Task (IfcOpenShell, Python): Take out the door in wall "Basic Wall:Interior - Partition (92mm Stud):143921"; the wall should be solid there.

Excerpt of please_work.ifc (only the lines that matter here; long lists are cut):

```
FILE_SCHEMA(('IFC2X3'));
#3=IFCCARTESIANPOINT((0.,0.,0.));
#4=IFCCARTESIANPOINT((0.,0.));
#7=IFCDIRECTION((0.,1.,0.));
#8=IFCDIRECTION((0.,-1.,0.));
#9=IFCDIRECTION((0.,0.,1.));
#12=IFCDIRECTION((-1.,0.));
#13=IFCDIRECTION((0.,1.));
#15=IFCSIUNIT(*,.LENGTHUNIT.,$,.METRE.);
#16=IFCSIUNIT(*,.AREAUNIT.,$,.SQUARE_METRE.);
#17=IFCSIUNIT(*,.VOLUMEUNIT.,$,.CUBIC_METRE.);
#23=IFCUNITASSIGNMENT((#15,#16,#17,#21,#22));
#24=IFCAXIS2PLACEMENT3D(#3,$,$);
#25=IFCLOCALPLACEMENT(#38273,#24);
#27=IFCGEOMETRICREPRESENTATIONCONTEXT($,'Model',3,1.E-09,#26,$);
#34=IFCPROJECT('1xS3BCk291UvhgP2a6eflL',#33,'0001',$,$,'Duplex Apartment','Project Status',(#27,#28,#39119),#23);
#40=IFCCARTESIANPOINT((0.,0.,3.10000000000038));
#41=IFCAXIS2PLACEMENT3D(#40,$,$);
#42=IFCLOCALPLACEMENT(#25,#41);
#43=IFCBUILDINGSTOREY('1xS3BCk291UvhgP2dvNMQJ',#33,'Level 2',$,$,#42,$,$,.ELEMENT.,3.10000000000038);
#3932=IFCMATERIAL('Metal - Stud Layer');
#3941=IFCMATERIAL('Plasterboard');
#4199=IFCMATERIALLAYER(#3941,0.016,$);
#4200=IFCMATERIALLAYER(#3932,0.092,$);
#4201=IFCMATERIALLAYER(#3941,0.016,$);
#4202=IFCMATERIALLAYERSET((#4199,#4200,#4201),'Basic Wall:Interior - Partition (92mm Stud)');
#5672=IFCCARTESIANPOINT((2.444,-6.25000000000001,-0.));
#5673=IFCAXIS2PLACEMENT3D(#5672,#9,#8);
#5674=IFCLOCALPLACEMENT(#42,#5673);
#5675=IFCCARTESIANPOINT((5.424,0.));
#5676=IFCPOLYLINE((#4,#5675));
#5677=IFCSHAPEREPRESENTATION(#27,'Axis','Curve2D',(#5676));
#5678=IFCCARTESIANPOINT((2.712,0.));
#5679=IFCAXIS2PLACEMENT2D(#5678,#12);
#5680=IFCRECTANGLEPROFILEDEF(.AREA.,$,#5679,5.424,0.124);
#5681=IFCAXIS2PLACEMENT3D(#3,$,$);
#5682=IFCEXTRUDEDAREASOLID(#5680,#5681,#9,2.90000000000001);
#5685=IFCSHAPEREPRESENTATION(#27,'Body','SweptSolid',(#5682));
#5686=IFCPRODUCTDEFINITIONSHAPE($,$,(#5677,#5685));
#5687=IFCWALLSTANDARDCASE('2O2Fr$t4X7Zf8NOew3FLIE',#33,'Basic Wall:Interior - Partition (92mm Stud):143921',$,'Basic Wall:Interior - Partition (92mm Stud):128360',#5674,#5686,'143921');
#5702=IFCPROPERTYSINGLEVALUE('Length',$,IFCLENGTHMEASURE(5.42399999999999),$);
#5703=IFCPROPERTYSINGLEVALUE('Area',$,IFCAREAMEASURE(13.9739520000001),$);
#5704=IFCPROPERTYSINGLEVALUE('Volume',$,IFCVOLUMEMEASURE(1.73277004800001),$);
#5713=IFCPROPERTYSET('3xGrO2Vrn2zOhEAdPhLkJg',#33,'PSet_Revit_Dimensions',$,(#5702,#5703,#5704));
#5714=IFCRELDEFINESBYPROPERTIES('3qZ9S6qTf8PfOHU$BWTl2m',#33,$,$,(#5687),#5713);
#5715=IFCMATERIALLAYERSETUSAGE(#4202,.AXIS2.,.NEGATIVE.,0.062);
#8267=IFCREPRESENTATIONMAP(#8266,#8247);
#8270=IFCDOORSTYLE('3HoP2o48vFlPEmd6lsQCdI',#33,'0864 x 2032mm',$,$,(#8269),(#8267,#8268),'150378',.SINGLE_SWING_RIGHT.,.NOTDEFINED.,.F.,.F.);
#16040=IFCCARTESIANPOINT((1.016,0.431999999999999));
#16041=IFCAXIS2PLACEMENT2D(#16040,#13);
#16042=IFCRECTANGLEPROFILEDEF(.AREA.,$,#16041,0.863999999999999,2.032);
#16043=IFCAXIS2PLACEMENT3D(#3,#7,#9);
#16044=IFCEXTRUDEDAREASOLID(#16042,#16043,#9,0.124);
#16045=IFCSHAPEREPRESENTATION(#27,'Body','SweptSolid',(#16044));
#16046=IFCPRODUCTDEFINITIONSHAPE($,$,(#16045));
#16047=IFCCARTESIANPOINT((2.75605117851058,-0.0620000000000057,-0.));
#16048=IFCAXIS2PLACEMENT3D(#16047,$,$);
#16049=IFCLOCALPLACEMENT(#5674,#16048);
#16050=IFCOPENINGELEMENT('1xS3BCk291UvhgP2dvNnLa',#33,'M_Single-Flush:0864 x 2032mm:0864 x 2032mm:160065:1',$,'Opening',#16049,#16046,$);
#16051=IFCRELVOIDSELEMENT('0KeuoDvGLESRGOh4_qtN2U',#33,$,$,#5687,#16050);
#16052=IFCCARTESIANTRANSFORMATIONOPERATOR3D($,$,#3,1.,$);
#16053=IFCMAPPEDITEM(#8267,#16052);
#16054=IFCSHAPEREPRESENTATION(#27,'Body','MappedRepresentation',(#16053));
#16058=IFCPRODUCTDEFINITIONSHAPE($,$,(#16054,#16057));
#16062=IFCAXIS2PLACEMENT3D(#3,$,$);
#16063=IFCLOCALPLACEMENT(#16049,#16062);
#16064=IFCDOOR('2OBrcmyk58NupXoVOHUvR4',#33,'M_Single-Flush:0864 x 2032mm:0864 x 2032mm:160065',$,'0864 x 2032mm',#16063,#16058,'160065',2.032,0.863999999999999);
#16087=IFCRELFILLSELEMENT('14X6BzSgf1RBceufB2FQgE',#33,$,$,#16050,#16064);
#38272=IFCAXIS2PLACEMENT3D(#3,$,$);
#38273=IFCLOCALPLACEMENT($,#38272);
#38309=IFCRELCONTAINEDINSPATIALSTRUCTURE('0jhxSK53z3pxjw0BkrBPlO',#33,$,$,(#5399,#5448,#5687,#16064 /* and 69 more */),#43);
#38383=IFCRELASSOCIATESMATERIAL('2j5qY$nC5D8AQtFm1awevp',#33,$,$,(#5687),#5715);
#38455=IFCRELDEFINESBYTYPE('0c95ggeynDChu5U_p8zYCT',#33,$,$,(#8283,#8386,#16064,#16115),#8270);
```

```python
import ifcopenshell
import ifcopenshell.api.feature
import ifcopenshell.api.pset
import ifcopenshell.api.root
import ifcopenshell.geom
import ifcopenshell.util.element
import ifcopenshell.util.shape
import ifcopenshell.util.unit

model = ifcopenshell.open("please_work.ifc")
area_scale = ifcopenshell.util.unit.calculate_unit_scale(model, "AREAUNIT")
volume_scale = ifcopenshell.util.unit.calculate_unit_scale(model, "VOLUMEUNIT")
settings = ifcopenshell.geom.settings()


def volume(element):
    """Net volume in cubic metres, openings subtracted."""
    shape = ifcopenshell.geom.create_shape(settings, element)
    return ifcopenshell.util.shape.get_volume(shape.geometry)


door = model.by_guid("2OBrcmyk58NupXoVOHUvR4")
opening = door.FillsVoids[0].RelatingOpeningElement
wall = opening.VoidsElements[0].RelatingBuildingElement
before = volume(wall)

ifcopenshell.api.root.remove_product(model, product=door)
ifcopenshell.api.feature.remove_feature(model, feature=opening)

after = volume(wall)
thickness = 0.124  # wall thickness in metres

# Update the wall's stored quantities.
pset = model.by_id(ifcopenshell.util.element.get_pset(wall, "PSet_Revit_Dimensions", should_inherit=False)["id"])
ifcopenshell.api.pset.edit_pset(model, pset=pset, properties={
    "Area": model.create_entity("IfcAreaMeasure", after / thickness / area_scale),
    "Volume": model.create_entity("IfcVolumeMeasure", after / volume_scale),
})

print(f"wall volume {before:.3f} -> {after:.3f} m3")

model.write("please_work_rev.ifc")
```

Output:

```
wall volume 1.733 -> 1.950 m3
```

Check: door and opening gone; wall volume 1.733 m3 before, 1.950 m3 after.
